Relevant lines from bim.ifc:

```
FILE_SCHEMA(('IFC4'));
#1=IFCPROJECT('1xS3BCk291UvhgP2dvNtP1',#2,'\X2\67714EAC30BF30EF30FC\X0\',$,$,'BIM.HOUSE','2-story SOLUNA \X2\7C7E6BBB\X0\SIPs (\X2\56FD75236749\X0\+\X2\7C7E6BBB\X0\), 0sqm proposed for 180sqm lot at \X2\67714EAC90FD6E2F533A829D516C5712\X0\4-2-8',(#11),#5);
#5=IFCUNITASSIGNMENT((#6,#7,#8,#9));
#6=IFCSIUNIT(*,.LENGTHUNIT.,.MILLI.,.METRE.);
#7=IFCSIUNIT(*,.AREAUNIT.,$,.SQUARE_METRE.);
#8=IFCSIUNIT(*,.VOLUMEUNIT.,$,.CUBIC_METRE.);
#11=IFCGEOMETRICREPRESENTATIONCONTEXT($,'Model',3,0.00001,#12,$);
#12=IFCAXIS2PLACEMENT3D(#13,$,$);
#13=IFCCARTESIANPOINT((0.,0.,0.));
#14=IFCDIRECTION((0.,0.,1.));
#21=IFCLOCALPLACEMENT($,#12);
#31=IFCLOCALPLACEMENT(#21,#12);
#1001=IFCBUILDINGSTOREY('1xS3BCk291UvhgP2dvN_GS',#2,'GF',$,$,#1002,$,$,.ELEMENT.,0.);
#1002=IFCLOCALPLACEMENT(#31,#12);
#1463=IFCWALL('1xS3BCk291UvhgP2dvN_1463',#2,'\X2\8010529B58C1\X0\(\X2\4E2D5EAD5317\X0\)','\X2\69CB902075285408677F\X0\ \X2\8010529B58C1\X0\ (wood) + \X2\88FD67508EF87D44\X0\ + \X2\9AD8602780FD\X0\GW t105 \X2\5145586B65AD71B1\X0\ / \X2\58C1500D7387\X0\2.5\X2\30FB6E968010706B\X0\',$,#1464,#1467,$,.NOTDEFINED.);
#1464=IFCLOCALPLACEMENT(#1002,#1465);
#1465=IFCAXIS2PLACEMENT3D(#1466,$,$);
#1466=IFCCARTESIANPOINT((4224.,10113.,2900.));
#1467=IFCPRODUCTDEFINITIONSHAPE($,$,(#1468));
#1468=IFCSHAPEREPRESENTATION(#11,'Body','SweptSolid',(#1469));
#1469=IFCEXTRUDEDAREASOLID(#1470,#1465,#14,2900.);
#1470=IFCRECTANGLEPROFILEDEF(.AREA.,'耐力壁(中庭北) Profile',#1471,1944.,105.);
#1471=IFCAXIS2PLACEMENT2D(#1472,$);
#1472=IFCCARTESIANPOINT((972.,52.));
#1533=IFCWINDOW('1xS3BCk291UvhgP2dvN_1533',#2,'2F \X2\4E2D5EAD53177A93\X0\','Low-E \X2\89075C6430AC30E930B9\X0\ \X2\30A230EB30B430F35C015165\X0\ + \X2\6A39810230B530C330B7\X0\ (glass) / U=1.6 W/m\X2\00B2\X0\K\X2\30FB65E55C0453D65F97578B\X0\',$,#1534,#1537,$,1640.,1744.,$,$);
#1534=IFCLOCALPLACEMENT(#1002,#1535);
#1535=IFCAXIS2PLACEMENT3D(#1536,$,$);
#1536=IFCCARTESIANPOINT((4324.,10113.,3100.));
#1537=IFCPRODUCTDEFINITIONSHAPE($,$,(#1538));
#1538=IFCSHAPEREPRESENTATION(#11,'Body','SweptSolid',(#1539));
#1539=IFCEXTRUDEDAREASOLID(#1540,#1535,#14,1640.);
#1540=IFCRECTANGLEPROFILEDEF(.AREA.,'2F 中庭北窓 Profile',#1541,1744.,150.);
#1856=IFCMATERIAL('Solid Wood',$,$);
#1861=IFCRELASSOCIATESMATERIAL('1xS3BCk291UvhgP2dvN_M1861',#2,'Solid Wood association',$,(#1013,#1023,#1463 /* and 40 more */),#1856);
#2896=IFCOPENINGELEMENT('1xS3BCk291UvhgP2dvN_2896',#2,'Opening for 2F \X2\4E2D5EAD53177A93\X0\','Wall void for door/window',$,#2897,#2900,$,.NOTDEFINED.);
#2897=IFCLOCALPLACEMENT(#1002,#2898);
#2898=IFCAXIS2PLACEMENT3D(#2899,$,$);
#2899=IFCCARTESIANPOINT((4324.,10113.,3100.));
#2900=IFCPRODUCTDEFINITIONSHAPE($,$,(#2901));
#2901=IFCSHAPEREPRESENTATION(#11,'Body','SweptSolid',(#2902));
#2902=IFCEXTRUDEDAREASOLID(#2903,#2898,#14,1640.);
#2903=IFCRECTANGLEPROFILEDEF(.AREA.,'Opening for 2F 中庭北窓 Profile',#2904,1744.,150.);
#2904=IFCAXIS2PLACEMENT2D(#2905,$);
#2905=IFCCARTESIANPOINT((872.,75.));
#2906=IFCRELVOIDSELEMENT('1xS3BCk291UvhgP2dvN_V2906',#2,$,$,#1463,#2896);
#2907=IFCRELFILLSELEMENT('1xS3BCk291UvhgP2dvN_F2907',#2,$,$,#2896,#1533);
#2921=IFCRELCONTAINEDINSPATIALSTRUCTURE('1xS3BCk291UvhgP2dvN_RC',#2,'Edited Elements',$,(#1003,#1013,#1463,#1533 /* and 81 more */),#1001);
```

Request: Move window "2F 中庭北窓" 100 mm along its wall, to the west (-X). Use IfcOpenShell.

```python
import ifcopenshell
import ifcopenshell.api.geometry
import ifcopenshell.util.placement
import ifcopenshell.util.unit

model = ifcopenshell.open("bim.ifc")
unit_scale = ifcopenshell.util.unit.calculate_unit_scale(model)

window = model.by_guid("1xS3BCk291UvhgP2dvN_1533")
opening = window.FillsVoids[0].RelatingOpeningElement
wall = opening.VoidsElements[0].RelatingBuildingElement

wall_matrix = ifcopenshell.util.placement.get_local_placement(wall.ObjectPlacement)
shift = wall_matrix[:3, 0] * -0.1 / unit_scale
before = ifcopenshell.util.placement.get_local_placement(window.ObjectPlacement)[:3, 3].copy()

# The window is not placed relative to its opening, so move both.
for product in (opening, window):
    matrix = ifcopenshell.util.placement.get_local_placement(product.ObjectPlacement)
    matrix[:3, 3] += shift
    ifcopenshell.api.geometry.edit_object_placement(model, product=product, matrix=matrix, is_si=False)

after = ifcopenshell.util.placement.get_local_placement(window.ObjectPlacement)[:3, 3]
print("window moved by", (after - before).round(3) + 0.0)

model.write("bim_rev.ifc")
```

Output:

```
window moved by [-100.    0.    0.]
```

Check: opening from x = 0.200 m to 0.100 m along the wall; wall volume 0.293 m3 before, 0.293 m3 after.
